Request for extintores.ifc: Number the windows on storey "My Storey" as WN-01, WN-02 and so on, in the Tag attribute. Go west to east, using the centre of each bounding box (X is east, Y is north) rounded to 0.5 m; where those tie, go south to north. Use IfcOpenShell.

First a look at what the model holds.

```python
import ifcopenshell
import ifcopenshell.util.element
import ifcopenshell.util.placement

model = ifcopenshell.open("extintores.ifc")
print(model.schema)
storey = next(s for s in model.by_type("IfcBuildingStorey") if s.Name == "My Storey")
windows = [e for e in ifcopenshell.util.element.get_decomposition(storey) if e.is_a("IfcWindow")]
for e in sorted(windows, key=lambda e: e.id()):
    origin = ifcopenshell.util.placement.get_local_placement(e.ObjectPlacement)[:3, 3]
    print(e.id(), e.Tag, e.Name, origin.round(2) + 0.0, sep=" | ")
```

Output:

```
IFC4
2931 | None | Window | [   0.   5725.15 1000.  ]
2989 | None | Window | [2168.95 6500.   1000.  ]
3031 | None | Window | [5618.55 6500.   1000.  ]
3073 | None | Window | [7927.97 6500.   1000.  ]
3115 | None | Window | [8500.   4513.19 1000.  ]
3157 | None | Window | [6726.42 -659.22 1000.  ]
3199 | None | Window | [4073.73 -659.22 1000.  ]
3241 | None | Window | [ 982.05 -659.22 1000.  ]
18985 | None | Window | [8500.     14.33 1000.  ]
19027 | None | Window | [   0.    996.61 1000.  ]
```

```python
import ifcopenshell
import ifcopenshell.geom
import ifcopenshell.util.element
import ifcopenshell.util.shape

model = ifcopenshell.open("extintores.ifc")
settings = ifcopenshell.geom.settings()
settings.set("use-world-coords", True)


def centre(element):
    shape = ifcopenshell.geom.create_shape(settings, element)
    return ifcopenshell.util.shape.get_bbox_centroid(shape.geometry)


storey = next(s for s in model.by_type("IfcBuildingStorey") if s.Name == "My Storey")
windows = [e for e in ifcopenshell.util.element.get_decomposition(storey) if e.is_a("IfcWindow")]

# Insertion points can sit at a corner or the storey origin, so sort by the geometry (in metres).
centres = {e: centre(e) for e in windows}
windows.sort(key=lambda e: (round(centres[e][0] / 0.5), centres[e][1]))

for i, e in enumerate(windows, start=1):
    number = f"WN-{i:02d}"
    e.Tag = number
    print(e.id(), number)

model.write("extintores_edited.ifc")
```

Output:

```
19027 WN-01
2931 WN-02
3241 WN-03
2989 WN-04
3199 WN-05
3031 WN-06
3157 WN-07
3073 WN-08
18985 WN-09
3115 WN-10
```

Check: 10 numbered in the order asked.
